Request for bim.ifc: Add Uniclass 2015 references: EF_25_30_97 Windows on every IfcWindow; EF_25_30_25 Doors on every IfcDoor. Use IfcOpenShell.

First a look at what the model holds.

```python
import ifcopenshell

model = ifcopenshell.open("bim.ifc")
print(model.schema)
print("classifications:", [c.Name for c in model.by_type("IfcClassification")])
for ifc_class in ("IfcDoor", "IfcRoof", "IfcStair", "IfcWall", "IfcWindow"):
    print(ifc_class, len(model.by_type(ifc_class)))
```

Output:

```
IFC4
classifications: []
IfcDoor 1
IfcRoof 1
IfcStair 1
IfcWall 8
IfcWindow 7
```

```python
import ifcopenshell
import ifcopenshell.api.classification

model = ifcopenshell.open("bim.ifc")

system = ifcopenshell.api.classification.add_classification(model, classification="Uniclass 2015")

codes = {
    "IfcWindow": ("EF_25_30_97", "Windows"),
    "IfcDoor": ("EF_25_30_25", "Doors"),
}
for ifc_class, (code, name) in codes.items():
    products = model.by_type(ifc_class)
    ifcopenshell.api.classification.add_reference(
        model, products=products, classification=system, identification=code, name=name
    )
    print(code, len(products))

model.write("bim_edited.ifc")
```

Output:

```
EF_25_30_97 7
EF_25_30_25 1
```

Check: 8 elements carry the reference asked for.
